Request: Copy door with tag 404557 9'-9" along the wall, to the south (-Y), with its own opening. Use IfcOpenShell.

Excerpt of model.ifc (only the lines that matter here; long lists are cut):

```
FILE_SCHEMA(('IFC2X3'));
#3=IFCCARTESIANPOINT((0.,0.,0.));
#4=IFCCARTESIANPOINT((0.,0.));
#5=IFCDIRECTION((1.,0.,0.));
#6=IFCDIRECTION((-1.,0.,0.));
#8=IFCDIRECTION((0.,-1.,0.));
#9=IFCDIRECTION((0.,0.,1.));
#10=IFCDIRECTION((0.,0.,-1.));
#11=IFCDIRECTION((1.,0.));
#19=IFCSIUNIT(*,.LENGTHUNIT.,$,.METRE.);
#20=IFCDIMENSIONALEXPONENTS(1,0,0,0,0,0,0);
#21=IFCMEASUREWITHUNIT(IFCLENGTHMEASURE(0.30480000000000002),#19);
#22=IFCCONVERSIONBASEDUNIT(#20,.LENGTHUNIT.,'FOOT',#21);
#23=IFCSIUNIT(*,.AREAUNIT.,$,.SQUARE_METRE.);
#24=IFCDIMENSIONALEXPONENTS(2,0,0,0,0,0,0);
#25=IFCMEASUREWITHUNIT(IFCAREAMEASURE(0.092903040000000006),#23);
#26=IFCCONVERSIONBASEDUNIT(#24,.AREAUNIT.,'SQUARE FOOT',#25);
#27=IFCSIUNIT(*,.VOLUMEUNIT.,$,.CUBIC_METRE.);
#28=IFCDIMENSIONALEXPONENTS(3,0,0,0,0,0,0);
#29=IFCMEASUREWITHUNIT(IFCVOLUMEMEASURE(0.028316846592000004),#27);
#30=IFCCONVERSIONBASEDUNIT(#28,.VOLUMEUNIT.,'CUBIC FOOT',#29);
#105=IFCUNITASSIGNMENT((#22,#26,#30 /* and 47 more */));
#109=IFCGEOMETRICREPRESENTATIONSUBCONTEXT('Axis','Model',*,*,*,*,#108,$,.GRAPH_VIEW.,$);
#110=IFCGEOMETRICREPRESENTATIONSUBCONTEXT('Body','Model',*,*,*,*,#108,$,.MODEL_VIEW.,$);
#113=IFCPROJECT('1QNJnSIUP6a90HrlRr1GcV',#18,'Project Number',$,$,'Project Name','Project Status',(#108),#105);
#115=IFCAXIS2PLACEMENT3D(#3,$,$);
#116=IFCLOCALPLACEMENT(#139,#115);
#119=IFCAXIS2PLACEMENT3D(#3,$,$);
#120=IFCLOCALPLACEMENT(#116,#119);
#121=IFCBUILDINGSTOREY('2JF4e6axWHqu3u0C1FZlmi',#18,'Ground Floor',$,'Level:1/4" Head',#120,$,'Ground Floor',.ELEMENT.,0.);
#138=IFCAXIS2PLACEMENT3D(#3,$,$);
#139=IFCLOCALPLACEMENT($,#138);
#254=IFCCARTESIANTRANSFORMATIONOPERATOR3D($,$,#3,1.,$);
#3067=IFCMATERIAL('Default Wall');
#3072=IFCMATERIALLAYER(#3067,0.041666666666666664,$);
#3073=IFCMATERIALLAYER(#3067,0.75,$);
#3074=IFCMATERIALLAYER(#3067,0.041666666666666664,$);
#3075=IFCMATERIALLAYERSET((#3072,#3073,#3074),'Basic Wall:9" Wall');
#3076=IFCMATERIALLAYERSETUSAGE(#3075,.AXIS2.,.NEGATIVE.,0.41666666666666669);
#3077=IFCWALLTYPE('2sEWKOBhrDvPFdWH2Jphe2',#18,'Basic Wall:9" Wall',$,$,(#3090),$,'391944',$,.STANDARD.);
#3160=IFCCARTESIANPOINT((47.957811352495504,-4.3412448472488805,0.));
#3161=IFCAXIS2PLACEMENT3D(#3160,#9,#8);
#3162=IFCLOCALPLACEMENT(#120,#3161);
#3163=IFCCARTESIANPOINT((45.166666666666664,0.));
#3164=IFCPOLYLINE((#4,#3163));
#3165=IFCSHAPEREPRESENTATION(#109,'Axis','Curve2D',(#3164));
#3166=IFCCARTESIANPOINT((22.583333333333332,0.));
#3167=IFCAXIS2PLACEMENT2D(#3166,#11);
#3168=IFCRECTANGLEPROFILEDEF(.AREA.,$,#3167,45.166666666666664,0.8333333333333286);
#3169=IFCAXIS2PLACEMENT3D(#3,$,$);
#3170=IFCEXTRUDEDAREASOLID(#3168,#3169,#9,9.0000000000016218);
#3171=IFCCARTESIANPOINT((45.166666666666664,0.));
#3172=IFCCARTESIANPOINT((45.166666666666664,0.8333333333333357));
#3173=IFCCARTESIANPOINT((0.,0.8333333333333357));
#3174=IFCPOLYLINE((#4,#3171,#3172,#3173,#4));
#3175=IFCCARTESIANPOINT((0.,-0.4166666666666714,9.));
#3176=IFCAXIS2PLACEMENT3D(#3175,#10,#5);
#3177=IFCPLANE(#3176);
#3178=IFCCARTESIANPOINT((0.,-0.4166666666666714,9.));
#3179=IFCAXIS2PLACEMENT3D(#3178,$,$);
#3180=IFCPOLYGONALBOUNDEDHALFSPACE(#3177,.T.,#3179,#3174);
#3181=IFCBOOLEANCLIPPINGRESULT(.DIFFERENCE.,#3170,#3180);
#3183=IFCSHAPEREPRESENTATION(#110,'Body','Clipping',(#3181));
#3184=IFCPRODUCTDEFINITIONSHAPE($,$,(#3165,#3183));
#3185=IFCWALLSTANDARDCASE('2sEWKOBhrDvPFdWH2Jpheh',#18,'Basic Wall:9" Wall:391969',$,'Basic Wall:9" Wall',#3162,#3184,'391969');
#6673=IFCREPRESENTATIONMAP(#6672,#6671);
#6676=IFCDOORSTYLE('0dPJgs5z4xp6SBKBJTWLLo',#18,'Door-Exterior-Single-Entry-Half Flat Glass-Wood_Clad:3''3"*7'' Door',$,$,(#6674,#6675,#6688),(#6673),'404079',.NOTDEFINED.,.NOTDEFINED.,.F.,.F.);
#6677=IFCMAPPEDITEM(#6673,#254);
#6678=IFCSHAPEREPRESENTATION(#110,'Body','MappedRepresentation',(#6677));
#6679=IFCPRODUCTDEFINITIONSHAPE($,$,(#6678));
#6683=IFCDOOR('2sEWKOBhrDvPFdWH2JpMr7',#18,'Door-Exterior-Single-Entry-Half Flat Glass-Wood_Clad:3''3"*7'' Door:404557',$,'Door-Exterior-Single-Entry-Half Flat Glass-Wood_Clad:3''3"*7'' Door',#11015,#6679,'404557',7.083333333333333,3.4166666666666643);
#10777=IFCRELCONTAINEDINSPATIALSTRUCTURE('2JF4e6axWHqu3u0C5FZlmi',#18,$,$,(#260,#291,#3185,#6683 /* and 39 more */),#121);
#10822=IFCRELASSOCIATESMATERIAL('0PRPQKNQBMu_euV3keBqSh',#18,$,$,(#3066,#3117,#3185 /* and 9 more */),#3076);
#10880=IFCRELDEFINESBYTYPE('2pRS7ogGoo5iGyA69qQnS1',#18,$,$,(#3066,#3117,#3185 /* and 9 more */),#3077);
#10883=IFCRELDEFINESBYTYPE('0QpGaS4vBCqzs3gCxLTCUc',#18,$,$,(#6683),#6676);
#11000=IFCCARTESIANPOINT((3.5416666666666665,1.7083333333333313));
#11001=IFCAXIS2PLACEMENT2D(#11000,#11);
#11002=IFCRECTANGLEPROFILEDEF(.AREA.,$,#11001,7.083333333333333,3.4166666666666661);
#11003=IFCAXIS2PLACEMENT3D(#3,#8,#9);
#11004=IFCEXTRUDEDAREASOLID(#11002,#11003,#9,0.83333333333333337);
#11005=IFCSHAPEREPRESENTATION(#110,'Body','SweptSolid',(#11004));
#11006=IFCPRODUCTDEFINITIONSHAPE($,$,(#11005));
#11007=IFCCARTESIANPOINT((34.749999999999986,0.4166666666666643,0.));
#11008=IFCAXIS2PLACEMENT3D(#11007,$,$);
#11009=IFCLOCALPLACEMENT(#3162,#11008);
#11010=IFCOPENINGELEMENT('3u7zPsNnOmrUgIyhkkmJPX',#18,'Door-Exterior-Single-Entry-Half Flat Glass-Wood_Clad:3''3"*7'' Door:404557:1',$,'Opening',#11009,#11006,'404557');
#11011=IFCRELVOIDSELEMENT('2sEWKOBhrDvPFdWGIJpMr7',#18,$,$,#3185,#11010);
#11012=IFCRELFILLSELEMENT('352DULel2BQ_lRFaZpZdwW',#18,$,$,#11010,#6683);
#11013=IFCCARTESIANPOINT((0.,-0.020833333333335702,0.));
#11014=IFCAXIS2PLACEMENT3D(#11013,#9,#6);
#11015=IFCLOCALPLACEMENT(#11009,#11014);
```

```python
import ifcopenshell
import ifcopenshell.api.feature
import ifcopenshell.api.geometry
import ifcopenshell.api.root
import ifcopenshell.geom
import ifcopenshell.util.element
import ifcopenshell.util.placement
import ifcopenshell.util.shape
import ifcopenshell.util.unit

model = ifcopenshell.open("model.ifc")
unit_scale = ifcopenshell.util.unit.calculate_unit_scale(model)
settings = ifcopenshell.geom.settings()


def volume(element):
    """Net volume in cubic metres, openings subtracted."""
    shape = ifcopenshell.geom.create_shape(settings, element)
    return ifcopenshell.util.shape.get_volume(shape.geometry)


def reuse_history(source, copy):
    """copy_class also copies each property set's owner history, people and application; keep the originals."""
    for rel in copy.IsDefinedBy:
        if rel.is_a("IfcRelDefinesByProperties") and (history := rel.RelatingPropertyDefinition.OwnerHistory):
            rel.RelatingPropertyDefinition.OwnerHistory = source.OwnerHistory
            ifcopenshell.util.element.remove_deep2(model, history)


door = model.by_id(6683)
opening = door.FillsVoids[0].RelatingOpeningElement
wall = opening.VoidsElements[0].RelatingBuildingElement
before = volume(wall)
shift = ifcopenshell.util.placement.get_local_placement(wall.ObjectPlacement)[:3, 0] * 117 * 0.0254 / unit_scale

# copy_class copies the void relationship, type, container and properties, but no geometry.
new_opening = ifcopenshell.api.root.copy_class(model, product=opening)
new_opening.Representation = ifcopenshell.util.element.copy_deep(
    model, opening.Representation, exclude=["IfcGeometricRepresentationContext", "IfcRepresentationMap"]
)
new_opening.Name = 'Door-Exterior-Single-Entry-Half Flat Glass-Wood_Clad:3\'3"*7\' Door'
new_opening.Tag = None
new_door = ifcopenshell.api.root.copy_class(model, product=door)
new_door.Representation = ifcopenshell.util.element.copy_deep(
    model, door.Representation, exclude=["IfcGeometricRepresentationContext", "IfcRepresentationMap"]
)
new_door.Name = 'Door-Exterior-Single-Entry-Half Flat Glass-Wood_Clad:3\'3"*7\' Door'
new_door.Tag = None
reuse_history(door, new_door)
fills = ifcopenshell.api.feature.add_filling(model, opening=new_opening, element=new_door)
fills.OwnerHistory = new_door.OwnerHistory  # required in IFC2X3

for old, new in ((opening, new_opening), (door, new_door)):
    matrix = ifcopenshell.util.placement.get_local_placement(old.ObjectPlacement)
    matrix[:3, 3] += shift
    ifcopenshell.api.geometry.edit_object_placement(model, product=new, matrix=matrix, is_si=False)

after = volume(wall)

print(f"wall volume {before:.3f} -> {after:.3f} m3")

model.write("model_updated.ifc")
```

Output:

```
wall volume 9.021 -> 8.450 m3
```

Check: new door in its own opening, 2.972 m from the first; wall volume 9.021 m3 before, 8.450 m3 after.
